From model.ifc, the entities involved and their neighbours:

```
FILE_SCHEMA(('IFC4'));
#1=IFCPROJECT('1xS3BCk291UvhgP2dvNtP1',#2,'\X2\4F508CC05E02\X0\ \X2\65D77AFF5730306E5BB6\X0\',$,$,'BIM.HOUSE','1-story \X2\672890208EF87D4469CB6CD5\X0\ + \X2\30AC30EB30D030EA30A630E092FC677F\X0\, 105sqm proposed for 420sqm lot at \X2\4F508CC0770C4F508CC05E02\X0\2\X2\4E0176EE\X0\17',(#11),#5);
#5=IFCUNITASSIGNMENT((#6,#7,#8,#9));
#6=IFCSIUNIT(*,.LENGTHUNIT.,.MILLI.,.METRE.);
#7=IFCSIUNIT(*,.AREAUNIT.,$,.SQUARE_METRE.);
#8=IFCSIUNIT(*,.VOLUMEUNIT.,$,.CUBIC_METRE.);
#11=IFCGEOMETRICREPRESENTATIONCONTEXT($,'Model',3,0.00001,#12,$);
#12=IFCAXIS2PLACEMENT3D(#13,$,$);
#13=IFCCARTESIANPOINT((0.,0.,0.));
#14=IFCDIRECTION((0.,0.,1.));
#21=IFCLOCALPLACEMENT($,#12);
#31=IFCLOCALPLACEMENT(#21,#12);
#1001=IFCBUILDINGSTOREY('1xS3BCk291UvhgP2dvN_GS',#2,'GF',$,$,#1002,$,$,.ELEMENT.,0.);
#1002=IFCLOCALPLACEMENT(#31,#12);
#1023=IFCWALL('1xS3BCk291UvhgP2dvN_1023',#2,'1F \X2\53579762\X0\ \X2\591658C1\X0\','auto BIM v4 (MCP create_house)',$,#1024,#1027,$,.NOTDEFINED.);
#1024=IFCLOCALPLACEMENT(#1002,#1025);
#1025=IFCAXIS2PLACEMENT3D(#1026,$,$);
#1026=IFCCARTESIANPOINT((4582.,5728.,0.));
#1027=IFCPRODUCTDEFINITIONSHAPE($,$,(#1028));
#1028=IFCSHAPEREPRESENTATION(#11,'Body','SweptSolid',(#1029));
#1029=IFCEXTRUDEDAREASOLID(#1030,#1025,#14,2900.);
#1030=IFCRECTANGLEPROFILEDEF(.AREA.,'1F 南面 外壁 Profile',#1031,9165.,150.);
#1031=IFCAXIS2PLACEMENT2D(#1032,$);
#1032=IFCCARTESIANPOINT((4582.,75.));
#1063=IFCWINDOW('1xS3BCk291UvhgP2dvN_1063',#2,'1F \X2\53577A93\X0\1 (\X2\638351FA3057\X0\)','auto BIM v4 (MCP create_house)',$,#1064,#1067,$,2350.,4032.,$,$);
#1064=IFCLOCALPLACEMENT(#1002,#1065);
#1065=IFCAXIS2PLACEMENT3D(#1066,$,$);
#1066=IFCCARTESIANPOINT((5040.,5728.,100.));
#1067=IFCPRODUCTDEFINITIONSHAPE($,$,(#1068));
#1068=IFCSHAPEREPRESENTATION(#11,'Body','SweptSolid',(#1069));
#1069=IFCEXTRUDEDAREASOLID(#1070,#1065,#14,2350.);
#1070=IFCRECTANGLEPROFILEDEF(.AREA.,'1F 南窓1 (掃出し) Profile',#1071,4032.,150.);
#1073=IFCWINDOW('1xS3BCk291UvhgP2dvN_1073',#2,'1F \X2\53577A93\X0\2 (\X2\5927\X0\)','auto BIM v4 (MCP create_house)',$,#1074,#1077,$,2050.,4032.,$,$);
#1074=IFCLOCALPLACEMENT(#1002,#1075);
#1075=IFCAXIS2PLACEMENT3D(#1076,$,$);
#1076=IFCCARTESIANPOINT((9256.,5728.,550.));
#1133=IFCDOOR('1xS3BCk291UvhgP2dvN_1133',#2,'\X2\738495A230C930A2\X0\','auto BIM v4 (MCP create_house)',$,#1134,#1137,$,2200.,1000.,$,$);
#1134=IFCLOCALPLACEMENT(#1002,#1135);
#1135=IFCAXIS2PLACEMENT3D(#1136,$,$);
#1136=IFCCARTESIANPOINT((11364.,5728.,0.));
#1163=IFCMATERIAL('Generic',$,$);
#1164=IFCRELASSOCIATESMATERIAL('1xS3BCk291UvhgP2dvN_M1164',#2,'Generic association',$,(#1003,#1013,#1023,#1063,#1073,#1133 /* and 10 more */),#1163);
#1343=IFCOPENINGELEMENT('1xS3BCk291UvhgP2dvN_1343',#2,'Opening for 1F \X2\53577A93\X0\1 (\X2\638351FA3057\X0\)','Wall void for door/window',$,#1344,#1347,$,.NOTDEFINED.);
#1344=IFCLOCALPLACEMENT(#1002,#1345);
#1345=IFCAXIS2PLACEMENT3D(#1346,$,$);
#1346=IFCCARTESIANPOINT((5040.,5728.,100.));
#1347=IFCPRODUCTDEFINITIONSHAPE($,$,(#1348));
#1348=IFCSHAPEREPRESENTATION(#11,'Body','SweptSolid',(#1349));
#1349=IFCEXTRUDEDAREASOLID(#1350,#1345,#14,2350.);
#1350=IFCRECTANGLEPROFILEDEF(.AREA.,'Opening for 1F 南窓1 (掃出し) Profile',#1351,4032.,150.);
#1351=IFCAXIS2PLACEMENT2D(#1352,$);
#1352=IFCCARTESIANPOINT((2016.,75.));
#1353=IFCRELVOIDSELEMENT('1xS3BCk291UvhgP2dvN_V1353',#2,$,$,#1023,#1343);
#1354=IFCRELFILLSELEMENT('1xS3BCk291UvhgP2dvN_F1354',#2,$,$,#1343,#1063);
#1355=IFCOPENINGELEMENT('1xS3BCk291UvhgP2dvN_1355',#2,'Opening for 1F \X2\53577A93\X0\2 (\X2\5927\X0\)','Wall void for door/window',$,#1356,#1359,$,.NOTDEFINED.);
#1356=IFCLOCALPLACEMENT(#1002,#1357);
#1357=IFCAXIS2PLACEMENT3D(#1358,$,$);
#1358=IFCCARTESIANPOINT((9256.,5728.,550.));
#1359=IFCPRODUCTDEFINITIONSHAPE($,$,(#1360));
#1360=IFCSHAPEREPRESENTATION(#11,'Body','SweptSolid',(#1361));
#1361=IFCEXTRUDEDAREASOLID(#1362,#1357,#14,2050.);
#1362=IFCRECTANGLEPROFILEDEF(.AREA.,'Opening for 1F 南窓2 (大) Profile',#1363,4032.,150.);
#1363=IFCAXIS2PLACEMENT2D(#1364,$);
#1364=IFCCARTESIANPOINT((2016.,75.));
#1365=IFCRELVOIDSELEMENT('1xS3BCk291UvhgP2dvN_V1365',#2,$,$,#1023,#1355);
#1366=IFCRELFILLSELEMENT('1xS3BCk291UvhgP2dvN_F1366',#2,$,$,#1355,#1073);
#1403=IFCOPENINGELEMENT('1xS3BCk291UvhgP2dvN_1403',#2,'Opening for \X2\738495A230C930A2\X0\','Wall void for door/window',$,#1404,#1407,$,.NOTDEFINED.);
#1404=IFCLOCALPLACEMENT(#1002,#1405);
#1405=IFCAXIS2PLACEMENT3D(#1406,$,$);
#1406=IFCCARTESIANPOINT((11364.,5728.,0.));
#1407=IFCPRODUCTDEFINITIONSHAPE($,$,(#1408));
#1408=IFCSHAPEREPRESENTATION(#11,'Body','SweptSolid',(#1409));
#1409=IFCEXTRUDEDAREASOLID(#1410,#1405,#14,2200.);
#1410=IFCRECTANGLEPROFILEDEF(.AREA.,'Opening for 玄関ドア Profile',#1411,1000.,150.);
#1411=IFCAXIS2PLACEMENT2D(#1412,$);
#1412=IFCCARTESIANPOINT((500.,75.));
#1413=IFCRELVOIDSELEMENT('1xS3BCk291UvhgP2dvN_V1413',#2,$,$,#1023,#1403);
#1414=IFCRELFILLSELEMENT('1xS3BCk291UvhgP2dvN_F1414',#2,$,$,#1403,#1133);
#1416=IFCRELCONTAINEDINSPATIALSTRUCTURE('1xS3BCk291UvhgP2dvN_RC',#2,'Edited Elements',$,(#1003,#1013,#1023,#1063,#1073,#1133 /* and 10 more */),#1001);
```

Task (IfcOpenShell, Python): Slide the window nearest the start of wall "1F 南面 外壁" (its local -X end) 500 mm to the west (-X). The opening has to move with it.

```python
import ifcopenshell
import ifcopenshell.api.geometry
import ifcopenshell.util.placement
import ifcopenshell.util.unit

model = ifcopenshell.open("model.ifc")
unit_scale = ifcopenshell.util.unit.calculate_unit_scale(model)

window = model.by_guid("1xS3BCk291UvhgP2dvN_1063")
opening = window.FillsVoids[0].RelatingOpeningElement
wall = opening.VoidsElements[0].RelatingBuildingElement

wall_matrix = ifcopenshell.util.placement.get_local_placement(wall.ObjectPlacement)
shift = wall_matrix[:3, 0] * -0.5 / unit_scale
before = ifcopenshell.util.placement.get_local_placement(window.ObjectPlacement)[:3, 3].copy()

# The window is not placed relative to its opening, so move both.
for product in (opening, window):
    matrix = ifcopenshell.util.placement.get_local_placement(product.ObjectPlacement)
    matrix[:3, 3] += shift
    ifcopenshell.api.geometry.edit_object_placement(model, product=product, matrix=matrix, is_si=False)

after = ifcopenshell.util.placement.get_local_placement(window.ObjectPlacement)[:3, 3]
print("window moved by", (after - before).round(3) + 0.0)

model.write("model-out.ifc")
```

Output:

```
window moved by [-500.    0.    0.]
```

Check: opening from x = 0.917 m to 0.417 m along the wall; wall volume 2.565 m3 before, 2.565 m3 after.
